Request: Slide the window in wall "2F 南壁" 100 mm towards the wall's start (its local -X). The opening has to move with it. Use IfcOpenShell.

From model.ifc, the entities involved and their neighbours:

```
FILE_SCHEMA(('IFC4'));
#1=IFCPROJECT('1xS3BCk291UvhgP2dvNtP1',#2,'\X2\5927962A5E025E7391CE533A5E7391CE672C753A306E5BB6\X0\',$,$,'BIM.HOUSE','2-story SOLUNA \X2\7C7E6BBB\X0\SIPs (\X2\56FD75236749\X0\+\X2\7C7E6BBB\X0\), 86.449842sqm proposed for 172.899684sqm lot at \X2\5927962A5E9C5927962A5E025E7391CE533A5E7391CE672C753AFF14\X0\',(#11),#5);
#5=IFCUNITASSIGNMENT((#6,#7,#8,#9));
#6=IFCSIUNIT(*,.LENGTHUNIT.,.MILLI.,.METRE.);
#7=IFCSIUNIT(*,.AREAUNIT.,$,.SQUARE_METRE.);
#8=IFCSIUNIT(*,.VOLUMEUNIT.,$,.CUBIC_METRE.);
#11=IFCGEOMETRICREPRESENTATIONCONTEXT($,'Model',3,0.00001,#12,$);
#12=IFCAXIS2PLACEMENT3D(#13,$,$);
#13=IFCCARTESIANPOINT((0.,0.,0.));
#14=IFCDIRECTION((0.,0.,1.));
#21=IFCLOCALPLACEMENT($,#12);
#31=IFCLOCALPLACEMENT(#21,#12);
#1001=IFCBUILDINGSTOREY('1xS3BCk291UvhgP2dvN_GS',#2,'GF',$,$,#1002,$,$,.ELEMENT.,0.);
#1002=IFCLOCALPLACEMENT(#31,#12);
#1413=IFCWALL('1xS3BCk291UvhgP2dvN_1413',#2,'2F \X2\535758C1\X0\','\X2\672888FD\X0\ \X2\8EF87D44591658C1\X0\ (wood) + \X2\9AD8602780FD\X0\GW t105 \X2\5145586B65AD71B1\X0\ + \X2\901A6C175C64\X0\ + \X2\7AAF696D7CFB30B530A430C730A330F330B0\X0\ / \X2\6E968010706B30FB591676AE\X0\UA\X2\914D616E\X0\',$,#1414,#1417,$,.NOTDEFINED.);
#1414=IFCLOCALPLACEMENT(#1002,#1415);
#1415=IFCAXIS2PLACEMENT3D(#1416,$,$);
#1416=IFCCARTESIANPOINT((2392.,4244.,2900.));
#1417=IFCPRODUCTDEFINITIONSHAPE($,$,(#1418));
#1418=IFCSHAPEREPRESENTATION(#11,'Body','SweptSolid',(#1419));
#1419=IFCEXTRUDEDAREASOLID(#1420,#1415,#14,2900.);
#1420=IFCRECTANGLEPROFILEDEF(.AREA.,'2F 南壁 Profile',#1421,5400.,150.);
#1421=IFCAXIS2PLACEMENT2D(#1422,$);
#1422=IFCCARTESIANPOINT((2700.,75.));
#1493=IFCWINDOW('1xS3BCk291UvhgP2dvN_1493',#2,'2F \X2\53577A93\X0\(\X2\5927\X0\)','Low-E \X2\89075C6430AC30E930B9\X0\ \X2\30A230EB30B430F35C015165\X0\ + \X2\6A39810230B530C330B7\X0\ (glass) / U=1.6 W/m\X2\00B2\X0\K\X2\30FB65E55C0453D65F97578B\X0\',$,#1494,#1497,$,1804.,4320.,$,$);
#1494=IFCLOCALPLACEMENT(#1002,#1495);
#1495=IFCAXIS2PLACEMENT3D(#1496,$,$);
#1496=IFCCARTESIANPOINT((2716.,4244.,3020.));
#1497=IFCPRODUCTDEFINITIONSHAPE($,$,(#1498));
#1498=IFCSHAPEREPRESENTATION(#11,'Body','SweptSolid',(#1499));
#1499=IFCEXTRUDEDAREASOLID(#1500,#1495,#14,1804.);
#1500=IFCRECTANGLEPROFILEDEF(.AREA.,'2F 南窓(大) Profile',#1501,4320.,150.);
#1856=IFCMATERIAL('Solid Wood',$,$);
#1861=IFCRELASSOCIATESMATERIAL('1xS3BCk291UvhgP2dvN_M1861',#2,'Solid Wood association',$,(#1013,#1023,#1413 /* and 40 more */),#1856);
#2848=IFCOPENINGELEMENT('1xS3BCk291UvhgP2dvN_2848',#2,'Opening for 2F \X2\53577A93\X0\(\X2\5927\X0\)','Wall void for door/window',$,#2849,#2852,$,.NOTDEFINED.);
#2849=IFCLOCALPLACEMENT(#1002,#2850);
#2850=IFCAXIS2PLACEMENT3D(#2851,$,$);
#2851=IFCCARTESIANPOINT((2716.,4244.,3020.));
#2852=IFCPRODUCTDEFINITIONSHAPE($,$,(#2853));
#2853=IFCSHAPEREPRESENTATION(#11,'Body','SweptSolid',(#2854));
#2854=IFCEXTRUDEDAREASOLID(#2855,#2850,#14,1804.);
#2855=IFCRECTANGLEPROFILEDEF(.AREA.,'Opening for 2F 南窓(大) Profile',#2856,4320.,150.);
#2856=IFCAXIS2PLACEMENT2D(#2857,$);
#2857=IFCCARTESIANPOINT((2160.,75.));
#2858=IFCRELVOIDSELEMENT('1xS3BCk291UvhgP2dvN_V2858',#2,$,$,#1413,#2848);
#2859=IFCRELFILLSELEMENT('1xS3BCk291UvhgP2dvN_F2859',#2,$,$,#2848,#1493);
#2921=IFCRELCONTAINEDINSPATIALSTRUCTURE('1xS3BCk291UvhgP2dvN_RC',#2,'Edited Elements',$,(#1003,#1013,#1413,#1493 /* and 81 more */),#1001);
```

```python
import ifcopenshell
import ifcopenshell.api.geometry
import ifcopenshell.util.placement
import ifcopenshell.util.unit

model = ifcopenshell.open("model.ifc")
unit_scale = ifcopenshell.util.unit.calculate_unit_scale(model)

window = model.by_guid("1xS3BCk291UvhgP2dvN_1493")
opening = window.FillsVoids[0].RelatingOpeningElement
wall = opening.VoidsElements[0].RelatingBuildingElement

wall_matrix = ifcopenshell.util.placement.get_local_placement(wall.ObjectPlacement)
shift = wall_matrix[:3, 0] * -0.1 / unit_scale
before = ifcopenshell.util.placement.get_local_placement(window.ObjectPlacement)[:3, 3].copy()

# The window is not placed relative to its opening, so move both.
for product in (opening, window):
    matrix = ifcopenshell.util.placement.get_local_placement(product.ObjectPlacement)
    matrix[:3, 3] += shift
    ifcopenshell.api.geometry.edit_object_placement(model, product=product, matrix=matrix, is_si=False)

after = ifcopenshell.util.placement.get_local_placement(window.ObjectPlacement)[:3, 3]
print("window moved by", (after - before).round(3) + 0.0)

model.write("model_edited.ifc")
```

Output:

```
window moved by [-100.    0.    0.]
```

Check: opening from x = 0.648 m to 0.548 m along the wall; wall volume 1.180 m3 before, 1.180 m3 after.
